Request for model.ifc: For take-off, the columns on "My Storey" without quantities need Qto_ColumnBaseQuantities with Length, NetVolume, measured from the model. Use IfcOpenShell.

First a look at what the model holds.

```python
import ifcopenshell
import ifcopenshell.util.element
import ifcopenshell.util.unit

model = ifcopenshell.open("model.ifc")
print(model.schema)
for unit_type in ("LENGTHUNIT", "AREAUNIT", "VOLUMEUNIT"):
    print(unit_type, ifcopenshell.util.unit.calculate_unit_scale(model, unit_type))
storey = next(s for s in model.by_type("IfcBuildingStorey") if s.Name == "My Storey")
columns = [e for e in ifcopenshell.util.element.get_decomposition(storey) if e.is_a("IfcColumn")]
for e in sorted(columns, key=lambda e: e.id()):
    print(e.id(), e.is_a(), e.Name, list(ifcopenshell.util.element.get_psets(e, qtos_only=True)), sep=" | ")
```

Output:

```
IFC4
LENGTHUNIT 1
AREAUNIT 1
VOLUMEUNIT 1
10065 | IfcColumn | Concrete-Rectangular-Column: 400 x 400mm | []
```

```python
import ifcopenshell
import ifcopenshell.api.pset
import ifcopenshell.geom
import ifcopenshell.util.element
import ifcopenshell.util.shape
import ifcopenshell.util.unit

model = ifcopenshell.open("model.ifc")
unit_scale = ifcopenshell.util.unit.calculate_unit_scale(model)
volume_scale = ifcopenshell.util.unit.calculate_unit_scale(model, "VOLUMEUNIT")
settings = ifcopenshell.geom.settings()

storey = next(s for s in model.by_type("IfcBuildingStorey") if s.Name == "My Storey")
columns = [e for e in ifcopenshell.util.element.get_decomposition(storey) if e.is_a("IfcColumn")]

for e in sorted(columns, key=lambda e: e.id()):
    if ifcopenshell.util.element.get_psets(e, qtos_only=True, should_inherit=False):
        continue
    # Geometry comes back in metres, in the element's own axes.
    shape = ifcopenshell.geom.create_shape(settings, e)
    values = {
        "Length": ifcopenshell.util.shape.get_z(shape.geometry) / unit_scale,
        "NetVolume": ifcopenshell.util.shape.get_volume(shape.geometry) / volume_scale,
    }
    qto = ifcopenshell.api.pset.add_qto(model, product=e, name="Qto_ColumnBaseQuantities")
    ifcopenshell.api.pset.edit_qto(model, qto=qto, properties=values)
    print(e.id(), {k: round(v, 3) for k, v in values.items()})

model.write("model_rev.ifc")
```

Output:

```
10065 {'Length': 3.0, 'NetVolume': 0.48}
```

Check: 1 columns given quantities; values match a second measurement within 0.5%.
